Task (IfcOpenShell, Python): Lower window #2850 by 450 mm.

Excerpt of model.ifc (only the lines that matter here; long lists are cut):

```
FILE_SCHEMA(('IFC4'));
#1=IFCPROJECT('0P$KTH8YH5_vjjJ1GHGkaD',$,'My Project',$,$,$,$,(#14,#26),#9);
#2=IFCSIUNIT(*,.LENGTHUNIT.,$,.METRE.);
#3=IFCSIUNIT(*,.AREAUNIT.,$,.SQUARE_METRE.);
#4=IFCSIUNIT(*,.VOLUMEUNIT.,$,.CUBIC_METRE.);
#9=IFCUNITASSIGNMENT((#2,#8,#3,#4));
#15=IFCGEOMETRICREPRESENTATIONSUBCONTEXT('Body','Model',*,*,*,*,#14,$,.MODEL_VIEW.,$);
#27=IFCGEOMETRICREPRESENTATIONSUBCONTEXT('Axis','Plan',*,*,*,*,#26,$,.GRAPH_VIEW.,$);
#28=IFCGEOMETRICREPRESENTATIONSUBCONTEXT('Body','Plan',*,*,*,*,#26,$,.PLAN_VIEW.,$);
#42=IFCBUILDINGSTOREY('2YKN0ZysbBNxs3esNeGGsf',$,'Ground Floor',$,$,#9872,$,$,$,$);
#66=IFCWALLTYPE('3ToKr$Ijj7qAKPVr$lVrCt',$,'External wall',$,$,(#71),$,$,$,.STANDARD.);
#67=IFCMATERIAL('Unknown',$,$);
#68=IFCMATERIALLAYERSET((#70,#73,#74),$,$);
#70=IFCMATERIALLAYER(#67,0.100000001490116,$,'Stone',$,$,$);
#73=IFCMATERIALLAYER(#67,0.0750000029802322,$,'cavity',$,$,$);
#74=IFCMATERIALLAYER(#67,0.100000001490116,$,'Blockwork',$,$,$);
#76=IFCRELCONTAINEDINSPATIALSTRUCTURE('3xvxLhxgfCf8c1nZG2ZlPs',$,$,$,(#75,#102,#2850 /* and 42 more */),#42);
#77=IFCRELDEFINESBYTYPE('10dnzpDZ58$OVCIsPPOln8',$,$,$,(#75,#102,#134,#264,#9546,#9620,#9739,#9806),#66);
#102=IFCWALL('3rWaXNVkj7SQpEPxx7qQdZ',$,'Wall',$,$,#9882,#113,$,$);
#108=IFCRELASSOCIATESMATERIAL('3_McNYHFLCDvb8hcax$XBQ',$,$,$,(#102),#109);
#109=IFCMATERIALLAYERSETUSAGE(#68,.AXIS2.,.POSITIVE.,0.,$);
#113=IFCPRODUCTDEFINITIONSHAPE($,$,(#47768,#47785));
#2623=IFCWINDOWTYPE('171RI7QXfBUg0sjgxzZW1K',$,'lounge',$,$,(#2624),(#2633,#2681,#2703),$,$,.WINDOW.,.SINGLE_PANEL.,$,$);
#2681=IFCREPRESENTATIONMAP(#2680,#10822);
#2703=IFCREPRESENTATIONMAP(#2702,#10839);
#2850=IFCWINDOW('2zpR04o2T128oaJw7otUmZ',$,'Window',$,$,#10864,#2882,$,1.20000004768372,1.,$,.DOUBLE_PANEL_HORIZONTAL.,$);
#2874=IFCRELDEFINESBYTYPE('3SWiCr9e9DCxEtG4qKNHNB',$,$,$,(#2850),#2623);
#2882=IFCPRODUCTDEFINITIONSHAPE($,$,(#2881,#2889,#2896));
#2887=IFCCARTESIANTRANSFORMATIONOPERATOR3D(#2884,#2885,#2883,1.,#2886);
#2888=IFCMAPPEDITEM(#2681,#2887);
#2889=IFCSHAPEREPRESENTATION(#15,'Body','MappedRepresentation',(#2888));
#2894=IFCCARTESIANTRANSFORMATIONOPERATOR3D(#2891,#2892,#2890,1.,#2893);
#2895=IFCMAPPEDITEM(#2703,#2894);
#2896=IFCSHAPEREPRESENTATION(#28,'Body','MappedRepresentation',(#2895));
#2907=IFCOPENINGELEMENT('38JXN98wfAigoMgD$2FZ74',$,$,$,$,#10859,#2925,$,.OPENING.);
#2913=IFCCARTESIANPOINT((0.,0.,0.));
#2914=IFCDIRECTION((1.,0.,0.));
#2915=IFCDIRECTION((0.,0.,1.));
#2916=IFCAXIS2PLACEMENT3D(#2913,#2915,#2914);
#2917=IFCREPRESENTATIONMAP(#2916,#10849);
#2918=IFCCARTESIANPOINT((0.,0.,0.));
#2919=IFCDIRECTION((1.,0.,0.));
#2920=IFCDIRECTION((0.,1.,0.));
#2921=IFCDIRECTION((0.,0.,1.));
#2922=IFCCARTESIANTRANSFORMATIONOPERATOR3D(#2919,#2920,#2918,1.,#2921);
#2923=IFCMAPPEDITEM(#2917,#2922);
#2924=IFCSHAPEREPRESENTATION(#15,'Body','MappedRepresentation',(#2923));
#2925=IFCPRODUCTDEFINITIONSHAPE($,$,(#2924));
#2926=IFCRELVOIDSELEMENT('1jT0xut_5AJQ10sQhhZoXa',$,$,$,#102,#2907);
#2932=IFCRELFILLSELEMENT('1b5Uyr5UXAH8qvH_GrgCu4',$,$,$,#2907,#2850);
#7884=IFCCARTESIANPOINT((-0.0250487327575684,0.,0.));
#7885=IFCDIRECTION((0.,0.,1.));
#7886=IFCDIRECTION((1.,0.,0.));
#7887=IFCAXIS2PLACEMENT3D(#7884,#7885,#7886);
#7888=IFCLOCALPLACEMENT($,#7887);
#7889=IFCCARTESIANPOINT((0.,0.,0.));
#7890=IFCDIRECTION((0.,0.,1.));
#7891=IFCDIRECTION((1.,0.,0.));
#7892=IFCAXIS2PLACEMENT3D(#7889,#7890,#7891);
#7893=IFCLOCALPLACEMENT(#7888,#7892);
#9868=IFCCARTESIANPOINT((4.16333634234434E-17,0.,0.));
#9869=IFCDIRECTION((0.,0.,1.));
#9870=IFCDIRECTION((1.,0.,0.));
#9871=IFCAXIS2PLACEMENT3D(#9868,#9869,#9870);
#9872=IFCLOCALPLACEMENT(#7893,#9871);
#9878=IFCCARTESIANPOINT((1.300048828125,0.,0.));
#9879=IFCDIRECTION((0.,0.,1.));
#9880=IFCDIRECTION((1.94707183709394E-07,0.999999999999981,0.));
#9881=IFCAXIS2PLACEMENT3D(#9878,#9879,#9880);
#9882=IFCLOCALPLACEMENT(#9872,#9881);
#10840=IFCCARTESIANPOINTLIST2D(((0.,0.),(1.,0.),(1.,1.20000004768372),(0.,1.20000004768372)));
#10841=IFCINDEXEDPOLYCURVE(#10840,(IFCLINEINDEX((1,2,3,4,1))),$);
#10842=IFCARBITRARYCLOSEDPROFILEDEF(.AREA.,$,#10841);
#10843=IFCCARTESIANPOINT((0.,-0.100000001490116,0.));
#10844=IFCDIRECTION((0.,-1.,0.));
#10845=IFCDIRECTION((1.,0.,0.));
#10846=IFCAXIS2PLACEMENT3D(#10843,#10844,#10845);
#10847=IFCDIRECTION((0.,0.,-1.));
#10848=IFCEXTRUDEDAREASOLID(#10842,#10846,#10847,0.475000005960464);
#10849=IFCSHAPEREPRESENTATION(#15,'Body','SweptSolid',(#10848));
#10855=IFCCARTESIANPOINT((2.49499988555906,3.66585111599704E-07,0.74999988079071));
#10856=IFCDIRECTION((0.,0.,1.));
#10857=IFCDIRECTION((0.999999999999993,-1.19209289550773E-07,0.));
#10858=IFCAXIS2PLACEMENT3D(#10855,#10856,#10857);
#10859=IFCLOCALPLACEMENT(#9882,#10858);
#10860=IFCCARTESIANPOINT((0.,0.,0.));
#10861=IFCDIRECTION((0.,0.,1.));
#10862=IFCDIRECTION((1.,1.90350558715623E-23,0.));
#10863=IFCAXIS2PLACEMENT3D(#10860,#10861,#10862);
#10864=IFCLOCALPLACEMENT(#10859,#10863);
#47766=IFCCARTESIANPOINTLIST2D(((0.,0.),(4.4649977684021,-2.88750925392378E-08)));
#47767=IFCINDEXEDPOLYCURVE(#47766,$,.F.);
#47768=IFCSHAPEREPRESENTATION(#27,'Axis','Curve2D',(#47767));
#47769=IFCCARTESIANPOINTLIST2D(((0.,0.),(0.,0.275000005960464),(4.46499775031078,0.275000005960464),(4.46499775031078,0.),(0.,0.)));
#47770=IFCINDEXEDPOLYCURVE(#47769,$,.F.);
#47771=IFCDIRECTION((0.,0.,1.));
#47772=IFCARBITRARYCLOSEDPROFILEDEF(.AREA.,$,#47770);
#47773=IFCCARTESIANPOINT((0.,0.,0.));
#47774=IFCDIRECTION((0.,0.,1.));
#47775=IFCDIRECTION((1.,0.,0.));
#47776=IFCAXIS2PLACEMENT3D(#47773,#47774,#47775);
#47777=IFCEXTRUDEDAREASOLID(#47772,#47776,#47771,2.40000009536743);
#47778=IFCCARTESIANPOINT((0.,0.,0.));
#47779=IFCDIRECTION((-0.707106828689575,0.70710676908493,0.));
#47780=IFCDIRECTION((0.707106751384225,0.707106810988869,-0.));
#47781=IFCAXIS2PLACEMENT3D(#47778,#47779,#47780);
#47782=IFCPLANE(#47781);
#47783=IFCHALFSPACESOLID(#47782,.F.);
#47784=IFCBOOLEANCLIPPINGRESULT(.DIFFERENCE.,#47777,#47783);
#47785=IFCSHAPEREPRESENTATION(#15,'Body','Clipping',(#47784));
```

```python
import numpy as np
import ifcopenshell
import ifcopenshell.api.geometry
import ifcopenshell.util.placement
import ifcopenshell.util.unit

model = ifcopenshell.open("model.ifc")
unit_scale = ifcopenshell.util.unit.calculate_unit_scale(model)

window = model.by_guid("2zpR04o2T128oaJw7otUmZ")
opening = window.FillsVoids[0].RelatingOpeningElement
dz = -0.45

shift = np.array([0.0, 0.0, dz])
# The window is placed relative to its opening, so it follows when the opening moves.
matrix = ifcopenshell.util.placement.get_local_placement(opening.ObjectPlacement)
matrix[:3, 3] += shift
ifcopenshell.api.geometry.edit_object_placement(
    model, product=opening, matrix=matrix, is_si=False, should_transform_children=True
)

print(f"moved by {dz * unit_scale:+.3f} m")

model.write("model_edited.ifc")
```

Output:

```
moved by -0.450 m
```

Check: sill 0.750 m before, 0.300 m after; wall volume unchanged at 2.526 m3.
